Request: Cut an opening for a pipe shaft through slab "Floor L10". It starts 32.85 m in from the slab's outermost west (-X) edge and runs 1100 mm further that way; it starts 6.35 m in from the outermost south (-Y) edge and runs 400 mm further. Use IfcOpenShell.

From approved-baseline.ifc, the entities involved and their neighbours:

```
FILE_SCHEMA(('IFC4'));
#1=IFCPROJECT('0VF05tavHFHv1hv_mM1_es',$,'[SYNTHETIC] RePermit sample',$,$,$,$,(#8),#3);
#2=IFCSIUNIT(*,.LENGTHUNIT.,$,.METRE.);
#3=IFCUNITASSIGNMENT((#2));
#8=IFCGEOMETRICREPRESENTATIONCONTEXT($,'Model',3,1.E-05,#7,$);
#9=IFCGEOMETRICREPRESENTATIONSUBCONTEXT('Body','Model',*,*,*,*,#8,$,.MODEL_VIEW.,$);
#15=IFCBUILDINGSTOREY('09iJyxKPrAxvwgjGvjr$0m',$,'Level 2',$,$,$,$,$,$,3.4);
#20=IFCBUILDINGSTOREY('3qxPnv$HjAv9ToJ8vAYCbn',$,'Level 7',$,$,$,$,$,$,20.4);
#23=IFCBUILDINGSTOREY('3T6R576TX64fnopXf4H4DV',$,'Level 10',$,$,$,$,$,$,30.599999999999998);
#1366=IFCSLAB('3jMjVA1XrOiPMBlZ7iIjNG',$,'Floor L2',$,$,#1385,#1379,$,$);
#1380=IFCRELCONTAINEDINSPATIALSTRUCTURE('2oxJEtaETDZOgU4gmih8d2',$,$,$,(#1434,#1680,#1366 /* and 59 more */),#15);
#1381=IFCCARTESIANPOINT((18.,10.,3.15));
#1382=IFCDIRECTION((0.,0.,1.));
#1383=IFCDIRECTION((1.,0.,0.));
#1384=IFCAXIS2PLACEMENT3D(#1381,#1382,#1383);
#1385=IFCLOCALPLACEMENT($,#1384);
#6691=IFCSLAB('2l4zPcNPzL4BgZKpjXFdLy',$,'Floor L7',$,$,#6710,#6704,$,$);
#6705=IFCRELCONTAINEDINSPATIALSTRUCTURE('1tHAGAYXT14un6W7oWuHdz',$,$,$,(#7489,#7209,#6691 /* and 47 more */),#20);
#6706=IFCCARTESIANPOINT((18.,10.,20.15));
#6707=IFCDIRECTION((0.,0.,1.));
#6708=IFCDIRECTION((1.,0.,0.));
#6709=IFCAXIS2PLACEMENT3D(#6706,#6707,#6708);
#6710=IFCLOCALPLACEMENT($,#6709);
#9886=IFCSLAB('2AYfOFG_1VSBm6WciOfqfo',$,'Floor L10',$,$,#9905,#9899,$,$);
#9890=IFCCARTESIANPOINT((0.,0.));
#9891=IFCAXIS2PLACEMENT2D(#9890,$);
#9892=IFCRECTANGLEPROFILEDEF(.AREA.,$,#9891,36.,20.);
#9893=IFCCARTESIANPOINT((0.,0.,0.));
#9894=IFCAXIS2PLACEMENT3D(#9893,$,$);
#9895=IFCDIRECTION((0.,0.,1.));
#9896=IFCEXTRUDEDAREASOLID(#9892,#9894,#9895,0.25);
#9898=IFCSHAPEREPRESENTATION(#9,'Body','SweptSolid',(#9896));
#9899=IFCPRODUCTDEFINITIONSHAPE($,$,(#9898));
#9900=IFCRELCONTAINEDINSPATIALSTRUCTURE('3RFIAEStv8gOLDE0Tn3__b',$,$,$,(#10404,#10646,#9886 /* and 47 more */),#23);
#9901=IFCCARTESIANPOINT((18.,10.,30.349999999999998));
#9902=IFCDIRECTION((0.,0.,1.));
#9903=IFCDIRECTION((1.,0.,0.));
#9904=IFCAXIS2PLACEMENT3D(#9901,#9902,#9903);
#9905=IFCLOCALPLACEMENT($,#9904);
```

```python
import numpy as np
import ifcopenshell
import ifcopenshell.api.feature
import ifcopenshell.api.geometry
import ifcopenshell.api.root
import ifcopenshell.geom
import ifcopenshell.util.placement
import ifcopenshell.util.representation
import ifcopenshell.util.shape
import ifcopenshell.util.unit

model = ifcopenshell.open("approved-baseline.ifc")
unit_scale = ifcopenshell.util.unit.calculate_unit_scale(model)
settings = ifcopenshell.geom.settings()


def volume(element):
    """Net volume in cubic metres, openings subtracted."""
    shape = ifcopenshell.geom.create_shape(settings, element)
    return ifcopenshell.util.shape.get_volume(shape.geometry)


slab = model.by_id(9886)
before = volume(slab)

# Extent in the slab's own axes, in metres. The edges named are its -X and -Y sides.
slab_shape = ifcopenshell.geom.create_shape(settings, slab)
vertices = ifcopenshell.util.shape.get_vertices(slab_shape.geometry)
x_min, y_min, bottom = vertices.min(axis=0)
top = vertices[:, 2].max()

opening = ifcopenshell.api.root.create_entity(model, ifc_class="IfcOpeningElement", name="Pipe shaft opening", predefined_type="OPENING")
context = ifcopenshell.util.representation.get_context(model, "Model", "Body", "MODEL_VIEW")
width, depth = 1.1, 0.4
outline = [(0.0, 0.0), (width, 0.0), (width, depth), (0.0, depth), (0.0, 0.0)]
# Overshoot both faces by 50 mm so the cut is clean.
shape = ifcopenshell.api.geometry.add_slab_representation(
    model, context=context, depth=top - bottom + 0.1, polyline=outline
)
ifcopenshell.api.geometry.assign_representation(model, product=opening, representation=shape)

matrix = ifcopenshell.util.placement.get_local_placement(slab.ObjectPlacement)
matrix[:, 3] = matrix @ np.append(np.array([x_min + 32.85, y_min + 6.35, bottom - 0.05]) / unit_scale, 1.0)
ifcopenshell.api.geometry.edit_object_placement(model, product=opening, matrix=matrix, is_si=False)
ifcopenshell.api.feature.add_feature(model, feature=opening, element=slab)

after = volume(slab)

print(f"slab volume {before:.3f} -> {after:.3f} m3")

model.write("approved-baseline_v2.ifc")
```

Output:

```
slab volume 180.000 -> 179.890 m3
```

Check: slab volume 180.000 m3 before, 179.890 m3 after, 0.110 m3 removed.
